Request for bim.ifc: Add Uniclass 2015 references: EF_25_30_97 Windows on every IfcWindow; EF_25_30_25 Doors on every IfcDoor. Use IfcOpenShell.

First a look at what the model holds.

```python
import ifcopenshell

model = ifcopenshell.open("bim.ifc")
print(model.schema)
print("classifications:", [c.Name for c in model.by_type("IfcClassification")])
for ifc_class in ("IfcDoor", "IfcRoof", "IfcStair", "IfcWall", "IfcWindow"):
    print(ifc_class, len(model.by_type(ifc_class)))
```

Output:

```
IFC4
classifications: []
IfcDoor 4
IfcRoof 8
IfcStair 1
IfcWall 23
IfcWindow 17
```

```python
import ifcopenshell
import ifcopenshell.api.classification

model = ifcopenshell.open("bim.ifc")

system = ifcopenshell.api.classification.add_classification(model, classification="Uniclass 2015")

codes = {
    "IfcWindow": ("EF_25_30_97", "Windows"),
    "IfcDoor": ("EF_25_30_25", "Doors"),
}
for ifc_class, (code, name) in codes.items():
    products = model.by_type(ifc_class)
    ifcopenshell.api.classification.add_reference(
        model, products=products, classification=system, identification=code, name=name
    )
    print(code, len(products))

model.write("bim_v2.ifc")
```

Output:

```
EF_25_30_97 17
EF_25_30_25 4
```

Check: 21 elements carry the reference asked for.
